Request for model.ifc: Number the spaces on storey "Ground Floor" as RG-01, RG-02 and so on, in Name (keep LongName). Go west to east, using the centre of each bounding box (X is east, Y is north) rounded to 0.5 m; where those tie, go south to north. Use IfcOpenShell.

First a look at what the model holds.

```python
import ifcopenshell
import ifcopenshell.util.element
import ifcopenshell.util.placement

model = ifcopenshell.open("model.ifc")
print(model.schema)
storey = next(s for s in model.by_type("IfcBuildingStorey") if s.Name == "Ground Floor")
spaces = [e for e in ifcopenshell.util.element.get_decomposition(storey) if e.is_a("IfcSpace")]
for e in sorted(spaces, key=lambda e: e.id()):
    origin = ifcopenshell.util.placement.get_local_placement(e.ObjectPlacement)[:3, 3]
    print(e.id(), e.Name, e.LongName, origin.round(2) + 0.0, sep=" | ")
```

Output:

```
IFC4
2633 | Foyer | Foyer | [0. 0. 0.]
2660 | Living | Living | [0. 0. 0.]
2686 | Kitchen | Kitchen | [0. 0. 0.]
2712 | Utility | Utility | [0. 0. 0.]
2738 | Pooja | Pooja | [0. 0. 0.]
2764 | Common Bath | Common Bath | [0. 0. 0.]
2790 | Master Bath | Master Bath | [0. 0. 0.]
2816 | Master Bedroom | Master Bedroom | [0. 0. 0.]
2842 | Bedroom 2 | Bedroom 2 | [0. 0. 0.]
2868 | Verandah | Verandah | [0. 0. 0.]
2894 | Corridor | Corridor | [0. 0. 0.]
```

```python
import ifcopenshell
import ifcopenshell.geom
import ifcopenshell.util.element
import ifcopenshell.util.shape

model = ifcopenshell.open("model.ifc")
settings = ifcopenshell.geom.settings()
settings.set("use-world-coords", True)


def centre(element):
    shape = ifcopenshell.geom.create_shape(settings, element)
    return ifcopenshell.util.shape.get_bbox_centroid(shape.geometry)


storey = next(s for s in model.by_type("IfcBuildingStorey") if s.Name == "Ground Floor")
spaces = [e for e in ifcopenshell.util.element.get_decomposition(storey) if e.is_a("IfcSpace")]

# Insertion points can sit at a corner or the storey origin, so sort by the geometry (in metres).
centres = {e: centre(e) for e in spaces}
spaces.sort(key=lambda e: (round(centres[e][0] / 0.5), centres[e][1]))

for i, e in enumerate(spaces, start=1):
    number = f"RG-{i:02d}"
    e.Name = number
    print(e.id(), number)

model.write("model_edited.ifc")
```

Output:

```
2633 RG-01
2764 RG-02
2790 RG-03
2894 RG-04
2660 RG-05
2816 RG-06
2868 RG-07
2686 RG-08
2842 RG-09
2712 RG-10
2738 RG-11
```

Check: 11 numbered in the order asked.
